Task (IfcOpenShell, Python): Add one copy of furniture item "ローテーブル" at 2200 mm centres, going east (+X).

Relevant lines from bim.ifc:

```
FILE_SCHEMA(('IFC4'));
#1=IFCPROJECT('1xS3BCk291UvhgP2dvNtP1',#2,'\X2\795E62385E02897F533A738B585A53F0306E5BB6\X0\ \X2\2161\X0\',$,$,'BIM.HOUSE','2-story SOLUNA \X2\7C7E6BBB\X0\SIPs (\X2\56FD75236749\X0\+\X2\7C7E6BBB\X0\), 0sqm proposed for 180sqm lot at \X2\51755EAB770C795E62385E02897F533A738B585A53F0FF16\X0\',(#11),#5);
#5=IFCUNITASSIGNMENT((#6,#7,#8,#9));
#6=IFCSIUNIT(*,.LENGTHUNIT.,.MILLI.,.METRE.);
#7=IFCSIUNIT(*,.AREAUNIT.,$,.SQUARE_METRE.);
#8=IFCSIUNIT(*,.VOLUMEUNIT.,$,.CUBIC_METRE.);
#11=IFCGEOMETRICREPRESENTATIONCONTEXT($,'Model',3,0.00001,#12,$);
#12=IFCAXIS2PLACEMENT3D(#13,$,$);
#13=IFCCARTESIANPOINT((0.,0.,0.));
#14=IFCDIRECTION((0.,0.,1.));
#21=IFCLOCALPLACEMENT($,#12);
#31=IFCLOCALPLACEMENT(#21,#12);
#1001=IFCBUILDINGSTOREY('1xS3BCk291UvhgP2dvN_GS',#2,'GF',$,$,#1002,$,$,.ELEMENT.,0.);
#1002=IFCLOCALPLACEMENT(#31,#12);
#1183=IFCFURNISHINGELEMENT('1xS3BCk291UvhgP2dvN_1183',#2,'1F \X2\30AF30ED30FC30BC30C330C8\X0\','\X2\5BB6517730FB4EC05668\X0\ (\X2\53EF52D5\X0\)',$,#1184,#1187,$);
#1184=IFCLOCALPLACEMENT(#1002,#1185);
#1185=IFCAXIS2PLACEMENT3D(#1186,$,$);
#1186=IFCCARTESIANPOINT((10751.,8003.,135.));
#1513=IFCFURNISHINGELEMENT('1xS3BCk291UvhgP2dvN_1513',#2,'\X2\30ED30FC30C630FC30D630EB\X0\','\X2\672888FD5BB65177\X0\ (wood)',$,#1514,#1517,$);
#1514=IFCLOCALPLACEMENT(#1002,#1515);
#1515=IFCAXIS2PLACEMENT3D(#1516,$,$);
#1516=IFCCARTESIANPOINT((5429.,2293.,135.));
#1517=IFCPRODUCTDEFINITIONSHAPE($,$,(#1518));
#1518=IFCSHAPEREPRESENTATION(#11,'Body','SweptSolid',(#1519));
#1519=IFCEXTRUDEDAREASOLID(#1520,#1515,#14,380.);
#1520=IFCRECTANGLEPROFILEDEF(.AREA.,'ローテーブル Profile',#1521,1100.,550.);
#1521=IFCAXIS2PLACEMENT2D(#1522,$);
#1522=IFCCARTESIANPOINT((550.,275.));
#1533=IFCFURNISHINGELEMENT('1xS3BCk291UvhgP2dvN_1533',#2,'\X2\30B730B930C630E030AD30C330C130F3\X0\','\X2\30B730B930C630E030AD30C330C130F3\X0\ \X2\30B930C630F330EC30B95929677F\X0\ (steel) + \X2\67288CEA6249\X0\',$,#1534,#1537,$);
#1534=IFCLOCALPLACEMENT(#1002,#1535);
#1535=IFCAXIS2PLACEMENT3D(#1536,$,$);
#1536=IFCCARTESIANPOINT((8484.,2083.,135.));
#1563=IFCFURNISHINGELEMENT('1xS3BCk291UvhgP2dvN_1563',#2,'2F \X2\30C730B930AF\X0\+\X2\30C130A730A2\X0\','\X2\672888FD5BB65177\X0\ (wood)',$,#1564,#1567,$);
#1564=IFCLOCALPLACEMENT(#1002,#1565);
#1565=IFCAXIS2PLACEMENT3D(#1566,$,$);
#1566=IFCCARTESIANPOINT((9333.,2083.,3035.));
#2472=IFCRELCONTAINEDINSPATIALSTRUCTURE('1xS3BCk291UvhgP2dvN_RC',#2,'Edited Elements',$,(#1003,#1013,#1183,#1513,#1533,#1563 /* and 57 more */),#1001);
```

```python
import numpy as np
import ifcopenshell
import ifcopenshell.api.geometry
import ifcopenshell.api.root
import ifcopenshell.util.element
import ifcopenshell.util.placement
import ifcopenshell.util.unit

model = ifcopenshell.open("bim.ifc")
unit_scale = ifcopenshell.util.unit.calculate_unit_scale(model)


def reuse_history(source, copy):
    """copy_class also copies each property set's owner history, people and application; keep the originals."""
    for rel in copy.IsDefinedBy:
        if rel.is_a("IfcRelDefinesByProperties") and (history := rel.RelatingPropertyDefinition.OwnerHistory):
            rel.RelatingPropertyDefinition.OwnerHistory = source.OwnerHistory
            ifcopenshell.util.element.remove_deep2(model, history)


source = model.by_guid("1xS3BCk291UvhgP2dvN_1513")
base = ifcopenshell.util.placement.get_local_placement(source.ObjectPlacement)
step = np.array([1.0, 0.0, 0.0]) * 2.2 / unit_scale

for i in range(1, 2):
    copy = ifcopenshell.api.root.copy_class(model, product=source)
    copy.Representation = ifcopenshell.util.element.copy_deep(
        model, source.Representation, exclude=["IfcGeometricRepresentationContext", "IfcRepresentationMap"]
    )
    reuse_history(source, copy)
    matrix = base.copy()
    matrix[:3, 3] += i * step
    print("added at", matrix[:3, 3].round(3) + 0.0)
    ifcopenshell.api.geometry.edit_object_placement(model, product=copy, matrix=matrix, is_si=False)

model.write("bim_rev.ifc")
```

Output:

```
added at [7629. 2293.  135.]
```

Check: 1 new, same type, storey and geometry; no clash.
